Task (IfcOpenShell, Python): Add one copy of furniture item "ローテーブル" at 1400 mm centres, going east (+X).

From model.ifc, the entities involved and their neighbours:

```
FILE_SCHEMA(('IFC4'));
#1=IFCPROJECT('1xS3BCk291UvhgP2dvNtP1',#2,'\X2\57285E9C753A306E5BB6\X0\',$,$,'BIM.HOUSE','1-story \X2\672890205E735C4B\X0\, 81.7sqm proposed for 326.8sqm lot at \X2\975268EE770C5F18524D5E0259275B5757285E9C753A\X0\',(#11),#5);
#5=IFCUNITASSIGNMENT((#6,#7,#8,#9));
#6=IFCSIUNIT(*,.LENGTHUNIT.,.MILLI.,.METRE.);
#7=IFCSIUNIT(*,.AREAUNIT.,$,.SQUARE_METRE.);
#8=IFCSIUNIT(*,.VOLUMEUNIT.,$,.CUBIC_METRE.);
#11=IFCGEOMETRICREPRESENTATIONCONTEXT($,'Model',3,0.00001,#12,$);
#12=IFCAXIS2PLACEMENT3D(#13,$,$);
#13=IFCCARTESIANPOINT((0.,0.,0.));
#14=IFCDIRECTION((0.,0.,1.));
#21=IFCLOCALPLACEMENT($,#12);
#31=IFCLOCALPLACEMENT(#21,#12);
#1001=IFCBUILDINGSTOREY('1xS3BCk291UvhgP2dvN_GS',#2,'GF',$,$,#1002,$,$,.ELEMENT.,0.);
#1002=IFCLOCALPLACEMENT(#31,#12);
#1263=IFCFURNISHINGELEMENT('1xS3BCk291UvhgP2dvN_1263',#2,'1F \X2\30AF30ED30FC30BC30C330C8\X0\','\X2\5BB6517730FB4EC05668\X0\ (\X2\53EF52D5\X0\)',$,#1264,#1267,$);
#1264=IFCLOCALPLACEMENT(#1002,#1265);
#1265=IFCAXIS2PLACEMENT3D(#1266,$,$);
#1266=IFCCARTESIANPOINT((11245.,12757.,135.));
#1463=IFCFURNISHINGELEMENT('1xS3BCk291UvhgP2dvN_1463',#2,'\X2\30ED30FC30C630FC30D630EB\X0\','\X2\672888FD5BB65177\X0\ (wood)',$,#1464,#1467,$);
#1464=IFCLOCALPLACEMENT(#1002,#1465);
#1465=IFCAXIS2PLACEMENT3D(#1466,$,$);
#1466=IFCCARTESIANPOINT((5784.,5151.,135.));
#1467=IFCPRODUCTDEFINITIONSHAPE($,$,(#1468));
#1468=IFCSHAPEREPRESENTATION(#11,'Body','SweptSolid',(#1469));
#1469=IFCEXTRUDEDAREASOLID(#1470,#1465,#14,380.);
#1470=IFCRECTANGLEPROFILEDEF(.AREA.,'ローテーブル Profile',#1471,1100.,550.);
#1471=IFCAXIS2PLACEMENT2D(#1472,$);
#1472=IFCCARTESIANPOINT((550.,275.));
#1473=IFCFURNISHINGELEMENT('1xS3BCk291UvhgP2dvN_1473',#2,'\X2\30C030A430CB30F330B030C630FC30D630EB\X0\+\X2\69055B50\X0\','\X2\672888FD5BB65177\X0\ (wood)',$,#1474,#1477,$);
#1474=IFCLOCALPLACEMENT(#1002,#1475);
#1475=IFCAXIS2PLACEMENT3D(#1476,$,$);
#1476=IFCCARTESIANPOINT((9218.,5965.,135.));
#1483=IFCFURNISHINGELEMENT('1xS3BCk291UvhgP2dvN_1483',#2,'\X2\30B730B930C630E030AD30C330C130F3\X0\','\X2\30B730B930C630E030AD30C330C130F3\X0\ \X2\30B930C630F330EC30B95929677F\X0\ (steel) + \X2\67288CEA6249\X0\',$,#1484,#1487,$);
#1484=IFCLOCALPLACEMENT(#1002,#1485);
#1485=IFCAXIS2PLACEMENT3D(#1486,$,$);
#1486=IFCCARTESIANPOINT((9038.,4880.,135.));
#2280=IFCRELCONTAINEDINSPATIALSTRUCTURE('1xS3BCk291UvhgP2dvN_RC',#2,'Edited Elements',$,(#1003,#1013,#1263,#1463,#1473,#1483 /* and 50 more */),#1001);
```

```python
import numpy as np
import ifcopenshell
import ifcopenshell.api.geometry
import ifcopenshell.api.root
import ifcopenshell.util.element
import ifcopenshell.util.placement

model = ifcopenshell.open("model.ifc")


def reuse_history(source, copy):
    """copy_class also copies each property set's owner history, people and application; keep the originals."""
    for rel in copy.IsDefinedBy:
        if rel.is_a("IfcRelDefinesByProperties") and (history := rel.RelatingPropertyDefinition.OwnerHistory):
            rel.RelatingPropertyDefinition.OwnerHistory = source.OwnerHistory
            ifcopenshell.util.element.remove_deep2(model, history)


source = model.by_id(1463)
base = ifcopenshell.util.placement.get_local_placement(source.ObjectPlacement)
step = np.array([1.0, 0.0, 0.0]) * 1400.0

for i in range(1, 2):
    copy = ifcopenshell.api.root.copy_class(model, product=source)
    copy.Representation = ifcopenshell.util.element.copy_deep(
        model, source.Representation, exclude=["IfcGeometricRepresentationContext", "IfcRepresentationMap"]
    )
    reuse_history(source, copy)
    matrix = base.copy()
    matrix[:3, 3] += i * step
    print("added at", matrix[:3, 3].round(3) + 0.0)
    ifcopenshell.api.geometry.edit_object_placement(model, product=copy, matrix=matrix, is_si=False)

model.write("model_updated.ifc")
```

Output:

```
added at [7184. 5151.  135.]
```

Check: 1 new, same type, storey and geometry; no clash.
